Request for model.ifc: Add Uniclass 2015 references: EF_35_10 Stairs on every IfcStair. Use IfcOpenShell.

First a look at what the model holds.

```python
import ifcopenshell

model = ifcopenshell.open("model.ifc")
print(model.schema)
print("classifications:", [c.Name for c in model.by_type("IfcClassification")])
for ifc_class in ("IfcDoor", "IfcRoof", "IfcStair", "IfcWall", "IfcWindow"):
    print(ifc_class, len(model.by_type(ifc_class)))
```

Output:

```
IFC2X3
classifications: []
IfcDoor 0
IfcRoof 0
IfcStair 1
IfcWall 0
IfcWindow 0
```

```python
import ifcopenshell
import ifcopenshell.api.classification

model = ifcopenshell.open("model.ifc")

# IFC2X3 requires Source and Edition and has no link from the project to the system.
system = model.create_entity("IfcClassification", Source="NBS", Edition="2015", Name="Uniclass 2015")

codes = {
    "IfcStair": ("EF_35_10", "Stairs"),
}
for ifc_class, (code, name) in codes.items():
    products = model.by_type(ifc_class)
    ifcopenshell.api.classification.add_reference(
        model, products=products, classification=system, identification=code, name=name
    )
    print(code, len(products))

model.write("model_updated.ifc")
```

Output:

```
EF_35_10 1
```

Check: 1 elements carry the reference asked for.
